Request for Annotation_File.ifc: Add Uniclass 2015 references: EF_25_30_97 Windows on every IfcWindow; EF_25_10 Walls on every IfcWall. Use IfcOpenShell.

First a look at what the model holds.

```python
import ifcopenshell

model = ifcopenshell.open("Annotation_File.ifc")
print(model.schema)
print("classifications:", [c.Name for c in model.by_type("IfcClassification")])
for ifc_class in ("IfcDoor", "IfcRoof", "IfcStair", "IfcWall", "IfcWindow"):
    print(ifc_class, len(model.by_type(ifc_class)))
```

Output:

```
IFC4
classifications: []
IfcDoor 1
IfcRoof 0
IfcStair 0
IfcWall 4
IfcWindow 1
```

```python
import ifcopenshell
import ifcopenshell.api.classification

model = ifcopenshell.open("Annotation_File.ifc")

system = ifcopenshell.api.classification.add_classification(model, classification="Uniclass 2015")

codes = {
    "IfcWindow": ("EF_25_30_97", "Windows"),
    "IfcWall": ("EF_25_10", "Walls"),
}
for ifc_class, (code, name) in codes.items():
    products = model.by_type(ifc_class)
    ifcopenshell.api.classification.add_reference(
        model, products=products, classification=system, identification=code, name=name
    )
    print(code, len(products))

model.write("Annotation_File_rev.ifc")
```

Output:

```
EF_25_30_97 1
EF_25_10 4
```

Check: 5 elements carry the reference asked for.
